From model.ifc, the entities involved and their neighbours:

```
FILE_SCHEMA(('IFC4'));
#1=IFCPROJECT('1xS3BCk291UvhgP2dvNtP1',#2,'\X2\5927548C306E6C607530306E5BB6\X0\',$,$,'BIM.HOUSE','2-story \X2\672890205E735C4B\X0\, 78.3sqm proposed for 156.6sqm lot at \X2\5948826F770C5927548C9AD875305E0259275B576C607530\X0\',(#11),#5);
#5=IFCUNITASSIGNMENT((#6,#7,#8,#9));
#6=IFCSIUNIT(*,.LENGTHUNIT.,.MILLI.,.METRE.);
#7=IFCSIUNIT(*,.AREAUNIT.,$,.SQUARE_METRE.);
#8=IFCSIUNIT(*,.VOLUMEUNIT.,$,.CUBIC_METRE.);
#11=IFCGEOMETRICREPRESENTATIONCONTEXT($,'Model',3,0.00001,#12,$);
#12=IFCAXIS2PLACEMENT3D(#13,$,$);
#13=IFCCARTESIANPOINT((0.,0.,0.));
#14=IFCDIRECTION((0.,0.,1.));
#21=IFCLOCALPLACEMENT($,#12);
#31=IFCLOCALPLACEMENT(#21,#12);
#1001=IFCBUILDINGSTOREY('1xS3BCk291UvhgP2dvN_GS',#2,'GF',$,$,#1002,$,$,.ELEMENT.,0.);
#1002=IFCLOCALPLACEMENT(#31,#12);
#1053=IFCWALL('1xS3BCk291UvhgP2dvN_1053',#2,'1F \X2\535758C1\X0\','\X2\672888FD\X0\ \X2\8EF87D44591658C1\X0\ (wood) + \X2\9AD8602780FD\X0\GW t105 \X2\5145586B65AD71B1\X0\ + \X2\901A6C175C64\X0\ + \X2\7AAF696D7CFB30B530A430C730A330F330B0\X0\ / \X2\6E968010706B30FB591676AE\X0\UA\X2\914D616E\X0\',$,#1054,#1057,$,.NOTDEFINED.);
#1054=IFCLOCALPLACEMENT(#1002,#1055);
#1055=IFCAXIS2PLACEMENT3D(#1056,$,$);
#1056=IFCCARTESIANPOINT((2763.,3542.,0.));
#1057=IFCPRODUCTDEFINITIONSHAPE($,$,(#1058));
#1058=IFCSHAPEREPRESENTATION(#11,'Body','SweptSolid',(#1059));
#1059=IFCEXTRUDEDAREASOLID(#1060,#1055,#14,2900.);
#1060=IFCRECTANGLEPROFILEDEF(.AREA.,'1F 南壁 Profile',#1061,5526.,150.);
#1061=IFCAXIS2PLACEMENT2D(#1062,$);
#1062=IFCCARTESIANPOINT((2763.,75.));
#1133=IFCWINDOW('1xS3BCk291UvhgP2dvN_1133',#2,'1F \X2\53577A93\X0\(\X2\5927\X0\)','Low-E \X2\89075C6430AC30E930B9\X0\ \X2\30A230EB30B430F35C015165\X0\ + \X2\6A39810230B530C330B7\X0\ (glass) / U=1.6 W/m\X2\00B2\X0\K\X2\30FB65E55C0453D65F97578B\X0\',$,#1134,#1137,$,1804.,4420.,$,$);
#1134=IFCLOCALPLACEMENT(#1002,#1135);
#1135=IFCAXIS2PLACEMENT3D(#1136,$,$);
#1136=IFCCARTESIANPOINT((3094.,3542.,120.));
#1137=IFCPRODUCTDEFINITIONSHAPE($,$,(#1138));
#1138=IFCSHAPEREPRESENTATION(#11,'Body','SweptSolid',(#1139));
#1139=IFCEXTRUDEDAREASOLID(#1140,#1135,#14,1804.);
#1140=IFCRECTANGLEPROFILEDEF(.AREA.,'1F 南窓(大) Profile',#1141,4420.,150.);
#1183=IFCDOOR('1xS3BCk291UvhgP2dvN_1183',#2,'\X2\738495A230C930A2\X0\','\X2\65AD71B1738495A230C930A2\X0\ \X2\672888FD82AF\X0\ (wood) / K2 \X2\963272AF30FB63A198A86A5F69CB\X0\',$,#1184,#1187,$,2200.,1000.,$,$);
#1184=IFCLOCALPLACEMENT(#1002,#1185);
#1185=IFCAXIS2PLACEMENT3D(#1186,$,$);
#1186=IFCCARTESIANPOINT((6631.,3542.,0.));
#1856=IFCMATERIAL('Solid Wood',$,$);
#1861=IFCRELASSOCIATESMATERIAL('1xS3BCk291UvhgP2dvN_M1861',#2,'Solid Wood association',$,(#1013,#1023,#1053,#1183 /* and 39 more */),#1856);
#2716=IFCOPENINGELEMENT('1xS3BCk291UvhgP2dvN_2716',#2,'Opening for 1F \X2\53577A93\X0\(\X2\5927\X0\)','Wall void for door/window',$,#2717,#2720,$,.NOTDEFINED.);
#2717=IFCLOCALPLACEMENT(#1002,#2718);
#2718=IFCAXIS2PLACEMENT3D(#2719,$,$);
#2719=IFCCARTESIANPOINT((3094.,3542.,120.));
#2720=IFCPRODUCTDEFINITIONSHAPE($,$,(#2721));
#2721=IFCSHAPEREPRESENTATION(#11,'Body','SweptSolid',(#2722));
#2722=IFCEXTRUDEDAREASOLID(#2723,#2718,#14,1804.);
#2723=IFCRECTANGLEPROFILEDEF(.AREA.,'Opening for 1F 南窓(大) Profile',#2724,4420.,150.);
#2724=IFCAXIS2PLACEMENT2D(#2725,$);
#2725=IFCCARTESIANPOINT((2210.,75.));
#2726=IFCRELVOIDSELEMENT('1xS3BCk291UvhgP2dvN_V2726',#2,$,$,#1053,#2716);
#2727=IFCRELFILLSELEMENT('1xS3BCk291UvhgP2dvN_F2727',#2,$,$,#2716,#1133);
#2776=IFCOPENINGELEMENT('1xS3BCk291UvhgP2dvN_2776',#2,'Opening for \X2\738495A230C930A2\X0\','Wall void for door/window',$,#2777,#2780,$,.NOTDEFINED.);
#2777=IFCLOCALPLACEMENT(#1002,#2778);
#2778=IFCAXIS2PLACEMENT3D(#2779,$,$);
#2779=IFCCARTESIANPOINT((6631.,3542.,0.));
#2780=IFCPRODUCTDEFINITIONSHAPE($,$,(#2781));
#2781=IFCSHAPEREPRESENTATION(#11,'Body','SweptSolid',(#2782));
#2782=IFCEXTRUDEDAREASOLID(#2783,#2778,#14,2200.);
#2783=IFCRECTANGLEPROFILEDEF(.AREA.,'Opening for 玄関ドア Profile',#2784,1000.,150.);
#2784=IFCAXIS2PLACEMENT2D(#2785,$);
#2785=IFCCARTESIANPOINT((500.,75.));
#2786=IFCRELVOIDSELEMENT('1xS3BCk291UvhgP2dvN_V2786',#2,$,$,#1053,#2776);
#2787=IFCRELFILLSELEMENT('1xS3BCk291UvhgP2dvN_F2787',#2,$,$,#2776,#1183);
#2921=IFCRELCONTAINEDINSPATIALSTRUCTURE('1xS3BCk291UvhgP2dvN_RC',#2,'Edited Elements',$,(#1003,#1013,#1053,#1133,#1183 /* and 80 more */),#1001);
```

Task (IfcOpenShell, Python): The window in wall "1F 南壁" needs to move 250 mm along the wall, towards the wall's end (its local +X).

```python
import ifcopenshell
import ifcopenshell.api.geometry
import ifcopenshell.util.placement
import ifcopenshell.util.unit

model = ifcopenshell.open("model.ifc")
unit_scale = ifcopenshell.util.unit.calculate_unit_scale(model)

window = model.by_guid("1xS3BCk291UvhgP2dvN_1133")
opening = window.FillsVoids[0].RelatingOpeningElement
wall = opening.VoidsElements[0].RelatingBuildingElement

wall_matrix = ifcopenshell.util.placement.get_local_placement(wall.ObjectPlacement)
shift = wall_matrix[:3, 0] * 0.25 / unit_scale
before = ifcopenshell.util.placement.get_local_placement(window.ObjectPlacement)[:3, 3].copy()

# The window is not placed relative to its opening, so move both.
for product in (opening, window):
    matrix = ifcopenshell.util.placement.get_local_placement(product.ObjectPlacement)
    matrix[:3, 3] += shift
    ifcopenshell.api.geometry.edit_object_placement(model, product=product, matrix=matrix, is_si=False)

after = ifcopenshell.util.placement.get_local_placement(window.ObjectPlacement)[:3, 3]
print("window moved by", (after - before).round(3) + 0.0)

model.write("model_edited.ifc")
```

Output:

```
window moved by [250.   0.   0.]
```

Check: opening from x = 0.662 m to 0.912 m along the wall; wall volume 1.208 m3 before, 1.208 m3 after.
